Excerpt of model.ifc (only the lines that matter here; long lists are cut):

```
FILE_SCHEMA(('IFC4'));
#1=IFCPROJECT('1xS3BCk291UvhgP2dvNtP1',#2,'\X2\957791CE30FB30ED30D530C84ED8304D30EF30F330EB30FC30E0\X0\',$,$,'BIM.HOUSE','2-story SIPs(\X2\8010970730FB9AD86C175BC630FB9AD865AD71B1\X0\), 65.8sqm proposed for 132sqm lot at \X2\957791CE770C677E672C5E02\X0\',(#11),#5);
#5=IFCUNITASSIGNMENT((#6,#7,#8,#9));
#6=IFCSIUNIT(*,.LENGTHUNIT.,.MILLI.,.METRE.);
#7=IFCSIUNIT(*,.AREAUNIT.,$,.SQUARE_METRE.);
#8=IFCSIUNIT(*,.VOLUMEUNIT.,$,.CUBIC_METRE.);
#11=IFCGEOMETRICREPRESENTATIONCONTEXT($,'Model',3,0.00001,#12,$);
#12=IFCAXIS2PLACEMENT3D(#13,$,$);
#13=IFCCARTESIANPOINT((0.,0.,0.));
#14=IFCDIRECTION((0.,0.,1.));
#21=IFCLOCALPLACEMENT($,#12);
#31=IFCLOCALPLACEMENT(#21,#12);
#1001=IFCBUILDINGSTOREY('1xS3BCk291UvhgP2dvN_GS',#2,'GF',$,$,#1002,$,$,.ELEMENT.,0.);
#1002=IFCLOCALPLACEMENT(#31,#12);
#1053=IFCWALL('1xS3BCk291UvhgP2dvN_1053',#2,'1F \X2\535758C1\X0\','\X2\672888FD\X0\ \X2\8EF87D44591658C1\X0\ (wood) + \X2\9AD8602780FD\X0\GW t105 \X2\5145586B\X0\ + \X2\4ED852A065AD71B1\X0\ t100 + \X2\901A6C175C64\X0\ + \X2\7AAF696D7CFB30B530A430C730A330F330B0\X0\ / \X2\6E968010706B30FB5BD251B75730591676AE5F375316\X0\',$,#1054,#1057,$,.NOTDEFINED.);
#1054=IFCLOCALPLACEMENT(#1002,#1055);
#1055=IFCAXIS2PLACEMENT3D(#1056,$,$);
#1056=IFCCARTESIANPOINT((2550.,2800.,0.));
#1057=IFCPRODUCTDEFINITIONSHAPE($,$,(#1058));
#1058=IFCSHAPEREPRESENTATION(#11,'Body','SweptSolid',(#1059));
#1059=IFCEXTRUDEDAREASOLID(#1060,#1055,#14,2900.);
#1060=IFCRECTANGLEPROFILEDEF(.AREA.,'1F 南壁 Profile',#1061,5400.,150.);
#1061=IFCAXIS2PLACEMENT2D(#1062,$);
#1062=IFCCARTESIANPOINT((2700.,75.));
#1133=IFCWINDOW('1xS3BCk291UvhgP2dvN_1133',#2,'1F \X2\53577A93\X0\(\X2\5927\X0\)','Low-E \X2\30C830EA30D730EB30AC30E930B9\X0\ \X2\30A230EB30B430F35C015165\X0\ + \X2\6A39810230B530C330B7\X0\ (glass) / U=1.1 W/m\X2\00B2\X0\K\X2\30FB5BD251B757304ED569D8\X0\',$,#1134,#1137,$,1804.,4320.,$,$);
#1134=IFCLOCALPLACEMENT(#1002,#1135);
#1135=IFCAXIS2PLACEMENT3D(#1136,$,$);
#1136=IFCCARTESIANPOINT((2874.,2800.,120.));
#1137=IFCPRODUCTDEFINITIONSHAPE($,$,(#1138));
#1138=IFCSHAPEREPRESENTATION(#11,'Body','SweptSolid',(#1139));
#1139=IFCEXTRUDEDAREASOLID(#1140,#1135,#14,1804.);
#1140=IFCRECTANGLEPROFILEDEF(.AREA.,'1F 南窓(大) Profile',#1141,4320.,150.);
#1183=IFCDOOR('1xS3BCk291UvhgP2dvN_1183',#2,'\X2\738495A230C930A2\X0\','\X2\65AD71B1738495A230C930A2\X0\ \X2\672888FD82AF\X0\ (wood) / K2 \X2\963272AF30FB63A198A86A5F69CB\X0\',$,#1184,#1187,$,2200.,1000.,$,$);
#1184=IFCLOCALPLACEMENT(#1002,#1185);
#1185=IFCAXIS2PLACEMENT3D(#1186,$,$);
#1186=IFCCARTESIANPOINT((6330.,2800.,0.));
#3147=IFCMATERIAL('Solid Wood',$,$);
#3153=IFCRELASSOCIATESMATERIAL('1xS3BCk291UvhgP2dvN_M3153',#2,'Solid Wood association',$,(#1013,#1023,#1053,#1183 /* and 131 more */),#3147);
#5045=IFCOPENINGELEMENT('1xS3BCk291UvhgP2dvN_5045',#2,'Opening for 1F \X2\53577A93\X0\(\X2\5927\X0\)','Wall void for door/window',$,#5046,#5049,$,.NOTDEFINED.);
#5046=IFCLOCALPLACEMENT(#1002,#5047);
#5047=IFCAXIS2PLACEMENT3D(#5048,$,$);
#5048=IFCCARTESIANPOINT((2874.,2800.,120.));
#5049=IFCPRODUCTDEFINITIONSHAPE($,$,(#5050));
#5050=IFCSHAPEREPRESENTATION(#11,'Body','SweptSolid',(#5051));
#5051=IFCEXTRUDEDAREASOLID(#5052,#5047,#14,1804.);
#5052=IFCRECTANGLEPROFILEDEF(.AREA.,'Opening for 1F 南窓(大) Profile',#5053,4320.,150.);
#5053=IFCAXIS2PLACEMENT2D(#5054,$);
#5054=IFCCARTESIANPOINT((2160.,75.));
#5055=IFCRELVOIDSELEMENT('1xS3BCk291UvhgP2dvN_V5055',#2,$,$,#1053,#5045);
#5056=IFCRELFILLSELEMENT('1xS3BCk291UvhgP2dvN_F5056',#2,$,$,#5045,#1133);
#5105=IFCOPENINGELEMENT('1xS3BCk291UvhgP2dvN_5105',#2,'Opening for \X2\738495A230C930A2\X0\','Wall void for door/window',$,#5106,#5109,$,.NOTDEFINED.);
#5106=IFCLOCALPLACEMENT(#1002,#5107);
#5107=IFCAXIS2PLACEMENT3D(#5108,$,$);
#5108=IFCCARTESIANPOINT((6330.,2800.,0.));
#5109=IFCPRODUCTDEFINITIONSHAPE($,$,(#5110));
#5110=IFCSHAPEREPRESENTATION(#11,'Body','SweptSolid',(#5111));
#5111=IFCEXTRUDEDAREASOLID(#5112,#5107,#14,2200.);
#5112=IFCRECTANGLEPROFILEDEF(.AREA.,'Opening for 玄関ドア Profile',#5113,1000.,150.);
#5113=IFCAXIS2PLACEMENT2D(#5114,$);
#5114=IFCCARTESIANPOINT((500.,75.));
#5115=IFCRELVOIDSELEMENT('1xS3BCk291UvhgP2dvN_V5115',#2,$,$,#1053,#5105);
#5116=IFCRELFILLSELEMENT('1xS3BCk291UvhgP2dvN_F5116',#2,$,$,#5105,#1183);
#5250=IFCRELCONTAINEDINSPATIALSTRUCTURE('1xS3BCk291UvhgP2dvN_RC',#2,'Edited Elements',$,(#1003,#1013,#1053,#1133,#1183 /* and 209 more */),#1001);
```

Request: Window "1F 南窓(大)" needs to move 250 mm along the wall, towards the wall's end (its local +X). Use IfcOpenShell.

```python
import ifcopenshell
import ifcopenshell.api.geometry
import ifcopenshell.util.placement

model = ifcopenshell.open("model.ifc")

window = model.by_guid("1xS3BCk291UvhgP2dvN_1133")
opening = window.FillsVoids[0].RelatingOpeningElement
wall = opening.VoidsElements[0].RelatingBuildingElement

wall_matrix = ifcopenshell.util.placement.get_local_placement(wall.ObjectPlacement)
shift = wall_matrix[:3, 0] * 250.0
before = ifcopenshell.util.placement.get_local_placement(window.ObjectPlacement)[:3, 3].copy()

# The window is not placed relative to its opening, so move both.
for product in (opening, window):
    matrix = ifcopenshell.util.placement.get_local_placement(product.ObjectPlacement)
    matrix[:3, 3] += shift
    ifcopenshell.api.geometry.edit_object_placement(model, product=product, matrix=matrix, is_si=False)

after = ifcopenshell.util.placement.get_local_placement(window.ObjectPlacement)[:3, 3]
print("window moved by", (after - before).round(3) + 0.0)

model.write("model_edited.ifc")
```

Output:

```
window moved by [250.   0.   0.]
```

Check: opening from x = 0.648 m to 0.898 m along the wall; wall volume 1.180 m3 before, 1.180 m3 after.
